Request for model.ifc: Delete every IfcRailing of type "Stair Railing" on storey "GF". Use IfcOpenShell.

First a look at what the model holds.

```python
import ifcopenshell
import ifcopenshell.util.element

model = ifcopenshell.open("model.ifc")
print(model.schema)
storey = next(s for s in model.by_type("IfcBuildingStorey") if s.Name == "GF")
railings = [e for e in ifcopenshell.util.element.get_decomposition(storey) if e.is_a("IfcRailing")]
seen = {}
for e in railings:
    element_type = ifcopenshell.util.element.get_type(e)
    name = element_type.Name if element_type not in (None, e) else None
    seen[name] = seen.get(name, 0) + 1
for name, count in sorted(seen.items(), key=str):
    print(count, "x", name)
```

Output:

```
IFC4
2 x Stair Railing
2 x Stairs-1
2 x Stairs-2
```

```python
import ifcopenshell
import ifcopenshell.api.root
import ifcopenshell.util.element

model = ifcopenshell.open("model.ifc")

storey = next(s for s in model.by_type("IfcBuildingStorey") if s.Name == "GF")
railings = [e for e in ifcopenshell.util.element.get_decomposition(storey) if e.is_a("IfcRailing")]
targets = [e for e in railings if (t := ifcopenshell.util.element.get_type(e)) not in (None, e) and t.Name == "Stair Railing"]

for e in targets:
    ifcopenshell.api.root.remove_product(model, product=e)
print(len(targets), "removed")

model.write("model_edited.ifc")
```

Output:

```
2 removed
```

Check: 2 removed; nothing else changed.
